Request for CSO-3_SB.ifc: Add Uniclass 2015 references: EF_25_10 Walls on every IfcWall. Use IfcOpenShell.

First a look at what the model holds.

```python
import ifcopenshell

model = ifcopenshell.open("CSO-3_SB.ifc")
print(model.schema)
print("classifications:", [c.Name for c in model.by_type("IfcClassification")])
for ifc_class in ("IfcDoor", "IfcRoof", "IfcStair", "IfcWall", "IfcWindow"):
    print(ifc_class, len(model.by_type(ifc_class)))
```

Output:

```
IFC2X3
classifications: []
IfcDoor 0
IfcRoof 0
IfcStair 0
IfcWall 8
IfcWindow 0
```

```python
import ifcopenshell
import ifcopenshell.api.classification

model = ifcopenshell.open("CSO-3_SB.ifc")

# IFC2X3 requires Source and Edition and has no link from the project to the system.
system = model.create_entity("IfcClassification", Source="NBS", Edition="2015", Name="Uniclass 2015")

codes = {
    "IfcWall": ("EF_25_10", "Walls"),
}
for ifc_class, (code, name) in codes.items():
    products = model.by_type(ifc_class)
    ifcopenshell.api.classification.add_reference(
        model, products=products, classification=system, identification=code, name=name
    )
    print(code, len(products))

model.write("CSO-3_SB_v2.ifc")
```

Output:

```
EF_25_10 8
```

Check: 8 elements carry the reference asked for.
